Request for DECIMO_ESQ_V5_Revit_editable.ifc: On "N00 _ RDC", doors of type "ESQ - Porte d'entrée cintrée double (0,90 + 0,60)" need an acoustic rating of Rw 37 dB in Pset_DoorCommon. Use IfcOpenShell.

First a look at what the model holds.

```python
import ifcopenshell
import ifcopenshell.util.element

model = ifcopenshell.open("DECIMO_ESQ_V5_Revit_editable.ifc")
print(model.schema)
storey = next(s for s in model.by_type("IfcBuildingStorey") if s.Name == "N00 _ RDC")
doors = [e for e in ifcopenshell.util.element.get_decomposition(storey) if e.is_a("IfcDoor")]
seen = {}
for e in doors:
    element_type = ifcopenshell.util.element.get_type(e)
    key = (element_type.Name if element_type != e and element_type else None, ifcopenshell.util.element.get_pset(e, "Pset_DoorCommon", "AcousticRating"))
    seen[key] = seen.get(key, 0) + 1
for (name, value), count in sorted(seen.items(), key=str):
    print(count, "x", name, "|", value)
```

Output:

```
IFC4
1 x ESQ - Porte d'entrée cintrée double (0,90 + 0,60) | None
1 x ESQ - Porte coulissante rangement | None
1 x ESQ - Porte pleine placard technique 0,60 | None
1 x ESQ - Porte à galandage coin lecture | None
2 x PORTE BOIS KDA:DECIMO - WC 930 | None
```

```python
import ifcopenshell
import ifcopenshell.api.pset
import ifcopenshell.util.element

model = ifcopenshell.open("DECIMO_ESQ_V5_Revit_editable.ifc")

storey = next(s for s in model.by_type("IfcBuildingStorey") if s.Name == "N00 _ RDC")
doors = [e for e in ifcopenshell.util.element.get_decomposition(storey) if e.is_a("IfcDoor")]

count = 0
for e in doors:
    element_type = ifcopenshell.util.element.get_type(e)
    if element_type in (None, e) or element_type.Name != "ESQ - Porte d'entrée cintrée double (0,90 + 0,60)":
        continue
    # add_pset returns the element's existing set when there is one.
    pset = ifcopenshell.api.pset.add_pset(model, product=e, name="Pset_DoorCommon")
    ifcopenshell.api.pset.edit_pset(model, pset=pset, properties={"AcousticRating": "Rw 37 dB"})
    count += 1

print(count, "doors updated")

model.write("DECIMO_ESQ_V5_Revit_editable_v2.ifc")
```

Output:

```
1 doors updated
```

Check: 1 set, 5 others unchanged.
